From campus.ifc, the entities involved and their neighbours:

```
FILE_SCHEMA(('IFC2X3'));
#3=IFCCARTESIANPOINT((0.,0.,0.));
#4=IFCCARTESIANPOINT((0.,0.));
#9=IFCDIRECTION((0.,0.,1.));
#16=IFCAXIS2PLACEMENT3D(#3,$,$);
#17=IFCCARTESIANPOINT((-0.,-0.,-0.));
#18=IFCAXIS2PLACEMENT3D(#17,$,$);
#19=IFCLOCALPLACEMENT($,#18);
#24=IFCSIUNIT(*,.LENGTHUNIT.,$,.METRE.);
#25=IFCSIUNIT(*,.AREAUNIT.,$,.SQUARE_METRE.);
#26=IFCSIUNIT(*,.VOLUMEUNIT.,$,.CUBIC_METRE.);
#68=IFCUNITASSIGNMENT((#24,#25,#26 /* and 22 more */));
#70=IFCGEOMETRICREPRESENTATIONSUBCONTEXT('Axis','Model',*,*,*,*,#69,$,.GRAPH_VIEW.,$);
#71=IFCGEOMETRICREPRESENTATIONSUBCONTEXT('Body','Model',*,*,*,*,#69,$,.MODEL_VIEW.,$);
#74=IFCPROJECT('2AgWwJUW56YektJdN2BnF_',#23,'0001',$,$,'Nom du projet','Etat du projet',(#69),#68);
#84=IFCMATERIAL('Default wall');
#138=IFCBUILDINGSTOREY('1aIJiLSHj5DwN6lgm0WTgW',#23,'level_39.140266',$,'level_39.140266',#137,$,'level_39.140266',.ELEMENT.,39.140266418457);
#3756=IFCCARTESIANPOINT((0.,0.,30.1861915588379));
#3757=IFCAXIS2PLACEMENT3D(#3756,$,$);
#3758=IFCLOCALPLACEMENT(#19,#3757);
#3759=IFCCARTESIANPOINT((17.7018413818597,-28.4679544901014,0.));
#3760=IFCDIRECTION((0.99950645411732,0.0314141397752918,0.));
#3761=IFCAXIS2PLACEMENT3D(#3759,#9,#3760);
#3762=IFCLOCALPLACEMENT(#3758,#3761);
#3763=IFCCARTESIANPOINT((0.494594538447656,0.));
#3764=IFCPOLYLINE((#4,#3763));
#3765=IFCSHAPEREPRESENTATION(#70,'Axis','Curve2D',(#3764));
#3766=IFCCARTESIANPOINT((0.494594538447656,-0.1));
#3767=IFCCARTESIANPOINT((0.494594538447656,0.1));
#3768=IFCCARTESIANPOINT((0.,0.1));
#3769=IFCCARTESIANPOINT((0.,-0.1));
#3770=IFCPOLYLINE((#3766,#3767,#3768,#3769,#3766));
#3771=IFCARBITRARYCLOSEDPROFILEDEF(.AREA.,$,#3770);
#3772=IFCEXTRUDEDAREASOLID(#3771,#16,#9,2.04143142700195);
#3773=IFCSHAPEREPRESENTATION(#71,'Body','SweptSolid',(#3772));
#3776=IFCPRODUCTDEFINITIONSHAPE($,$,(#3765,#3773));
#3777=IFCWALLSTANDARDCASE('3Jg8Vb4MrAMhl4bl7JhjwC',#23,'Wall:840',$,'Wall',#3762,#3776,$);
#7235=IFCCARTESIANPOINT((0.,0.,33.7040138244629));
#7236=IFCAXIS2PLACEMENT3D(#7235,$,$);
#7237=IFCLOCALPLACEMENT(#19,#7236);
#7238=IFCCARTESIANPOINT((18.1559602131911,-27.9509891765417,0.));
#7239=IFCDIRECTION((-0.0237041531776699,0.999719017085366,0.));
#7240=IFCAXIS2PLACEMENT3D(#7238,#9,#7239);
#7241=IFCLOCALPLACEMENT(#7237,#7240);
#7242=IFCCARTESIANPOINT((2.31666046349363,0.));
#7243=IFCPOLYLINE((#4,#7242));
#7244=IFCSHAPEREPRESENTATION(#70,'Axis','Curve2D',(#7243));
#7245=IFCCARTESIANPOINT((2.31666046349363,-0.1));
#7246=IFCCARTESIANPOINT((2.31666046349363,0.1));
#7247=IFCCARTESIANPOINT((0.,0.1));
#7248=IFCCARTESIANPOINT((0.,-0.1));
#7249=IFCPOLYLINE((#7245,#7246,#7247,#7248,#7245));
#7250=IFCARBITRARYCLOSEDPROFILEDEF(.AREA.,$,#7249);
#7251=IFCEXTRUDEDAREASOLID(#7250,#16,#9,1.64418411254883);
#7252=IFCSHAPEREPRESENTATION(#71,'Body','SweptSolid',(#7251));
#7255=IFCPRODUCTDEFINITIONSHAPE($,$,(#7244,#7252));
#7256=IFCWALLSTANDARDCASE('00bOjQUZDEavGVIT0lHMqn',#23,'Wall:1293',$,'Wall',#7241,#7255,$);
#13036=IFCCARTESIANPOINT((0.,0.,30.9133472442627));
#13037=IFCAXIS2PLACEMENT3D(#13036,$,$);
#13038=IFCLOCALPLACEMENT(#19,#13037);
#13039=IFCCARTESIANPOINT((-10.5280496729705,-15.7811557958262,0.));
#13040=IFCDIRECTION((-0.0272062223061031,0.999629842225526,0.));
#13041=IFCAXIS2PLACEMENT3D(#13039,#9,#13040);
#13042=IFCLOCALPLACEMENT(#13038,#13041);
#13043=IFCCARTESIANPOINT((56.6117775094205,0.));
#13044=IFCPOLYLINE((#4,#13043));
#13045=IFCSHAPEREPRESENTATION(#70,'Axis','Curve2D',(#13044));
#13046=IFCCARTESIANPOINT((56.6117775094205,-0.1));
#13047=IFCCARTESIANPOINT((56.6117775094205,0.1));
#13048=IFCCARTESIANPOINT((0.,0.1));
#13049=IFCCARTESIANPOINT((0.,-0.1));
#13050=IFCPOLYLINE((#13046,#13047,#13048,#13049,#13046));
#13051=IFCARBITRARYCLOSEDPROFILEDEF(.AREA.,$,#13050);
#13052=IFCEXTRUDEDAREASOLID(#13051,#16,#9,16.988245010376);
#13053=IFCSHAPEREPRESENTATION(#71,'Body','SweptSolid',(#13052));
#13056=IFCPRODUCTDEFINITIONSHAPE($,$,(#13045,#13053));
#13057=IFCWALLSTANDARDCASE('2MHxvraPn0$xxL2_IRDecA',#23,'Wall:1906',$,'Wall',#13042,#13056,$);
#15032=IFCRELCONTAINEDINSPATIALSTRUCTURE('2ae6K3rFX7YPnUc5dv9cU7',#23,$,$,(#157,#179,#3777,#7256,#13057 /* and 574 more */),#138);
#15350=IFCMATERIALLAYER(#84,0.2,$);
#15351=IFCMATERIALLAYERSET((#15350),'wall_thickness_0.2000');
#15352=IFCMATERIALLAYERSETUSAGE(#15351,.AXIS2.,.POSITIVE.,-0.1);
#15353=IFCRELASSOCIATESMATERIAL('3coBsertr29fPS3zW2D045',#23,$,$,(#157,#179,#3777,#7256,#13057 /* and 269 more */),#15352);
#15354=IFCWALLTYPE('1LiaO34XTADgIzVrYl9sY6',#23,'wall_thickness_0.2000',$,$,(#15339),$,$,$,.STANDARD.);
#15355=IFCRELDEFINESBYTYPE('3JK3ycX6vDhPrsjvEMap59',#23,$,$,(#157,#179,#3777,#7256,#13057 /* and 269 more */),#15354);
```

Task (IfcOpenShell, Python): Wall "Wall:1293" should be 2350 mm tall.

```python
import ifcopenshell
import ifcopenshell.geom
import ifcopenshell.util.representation
import ifcopenshell.util.shape

model = ifcopenshell.open("campus.ifc")
settings = ifcopenshell.geom.settings()


def volume(element):
    """Net volume in cubic metres, openings subtracted."""
    shape = ifcopenshell.geom.create_shape(settings, element)
    return ifcopenshell.util.shape.get_volume(shape.geometry)


wall = model.by_guid("00bOjQUZDEavGVIT0lHMqn")
before = volume(wall)

body = ifcopenshell.util.representation.get_representation(wall, "Model", "Body")
solid = body.Items[0]
old_height = solid.Depth
solid.Depth = 2.35
after = volume(wall)

print(f"height {old_height:g} -> {solid.Depth:g}, volume {before:.3f} -> {after:.3f} m3")

model.write("campus-out.ifc")
```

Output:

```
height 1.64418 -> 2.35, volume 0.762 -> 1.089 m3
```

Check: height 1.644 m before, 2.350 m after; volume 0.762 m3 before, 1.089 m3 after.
